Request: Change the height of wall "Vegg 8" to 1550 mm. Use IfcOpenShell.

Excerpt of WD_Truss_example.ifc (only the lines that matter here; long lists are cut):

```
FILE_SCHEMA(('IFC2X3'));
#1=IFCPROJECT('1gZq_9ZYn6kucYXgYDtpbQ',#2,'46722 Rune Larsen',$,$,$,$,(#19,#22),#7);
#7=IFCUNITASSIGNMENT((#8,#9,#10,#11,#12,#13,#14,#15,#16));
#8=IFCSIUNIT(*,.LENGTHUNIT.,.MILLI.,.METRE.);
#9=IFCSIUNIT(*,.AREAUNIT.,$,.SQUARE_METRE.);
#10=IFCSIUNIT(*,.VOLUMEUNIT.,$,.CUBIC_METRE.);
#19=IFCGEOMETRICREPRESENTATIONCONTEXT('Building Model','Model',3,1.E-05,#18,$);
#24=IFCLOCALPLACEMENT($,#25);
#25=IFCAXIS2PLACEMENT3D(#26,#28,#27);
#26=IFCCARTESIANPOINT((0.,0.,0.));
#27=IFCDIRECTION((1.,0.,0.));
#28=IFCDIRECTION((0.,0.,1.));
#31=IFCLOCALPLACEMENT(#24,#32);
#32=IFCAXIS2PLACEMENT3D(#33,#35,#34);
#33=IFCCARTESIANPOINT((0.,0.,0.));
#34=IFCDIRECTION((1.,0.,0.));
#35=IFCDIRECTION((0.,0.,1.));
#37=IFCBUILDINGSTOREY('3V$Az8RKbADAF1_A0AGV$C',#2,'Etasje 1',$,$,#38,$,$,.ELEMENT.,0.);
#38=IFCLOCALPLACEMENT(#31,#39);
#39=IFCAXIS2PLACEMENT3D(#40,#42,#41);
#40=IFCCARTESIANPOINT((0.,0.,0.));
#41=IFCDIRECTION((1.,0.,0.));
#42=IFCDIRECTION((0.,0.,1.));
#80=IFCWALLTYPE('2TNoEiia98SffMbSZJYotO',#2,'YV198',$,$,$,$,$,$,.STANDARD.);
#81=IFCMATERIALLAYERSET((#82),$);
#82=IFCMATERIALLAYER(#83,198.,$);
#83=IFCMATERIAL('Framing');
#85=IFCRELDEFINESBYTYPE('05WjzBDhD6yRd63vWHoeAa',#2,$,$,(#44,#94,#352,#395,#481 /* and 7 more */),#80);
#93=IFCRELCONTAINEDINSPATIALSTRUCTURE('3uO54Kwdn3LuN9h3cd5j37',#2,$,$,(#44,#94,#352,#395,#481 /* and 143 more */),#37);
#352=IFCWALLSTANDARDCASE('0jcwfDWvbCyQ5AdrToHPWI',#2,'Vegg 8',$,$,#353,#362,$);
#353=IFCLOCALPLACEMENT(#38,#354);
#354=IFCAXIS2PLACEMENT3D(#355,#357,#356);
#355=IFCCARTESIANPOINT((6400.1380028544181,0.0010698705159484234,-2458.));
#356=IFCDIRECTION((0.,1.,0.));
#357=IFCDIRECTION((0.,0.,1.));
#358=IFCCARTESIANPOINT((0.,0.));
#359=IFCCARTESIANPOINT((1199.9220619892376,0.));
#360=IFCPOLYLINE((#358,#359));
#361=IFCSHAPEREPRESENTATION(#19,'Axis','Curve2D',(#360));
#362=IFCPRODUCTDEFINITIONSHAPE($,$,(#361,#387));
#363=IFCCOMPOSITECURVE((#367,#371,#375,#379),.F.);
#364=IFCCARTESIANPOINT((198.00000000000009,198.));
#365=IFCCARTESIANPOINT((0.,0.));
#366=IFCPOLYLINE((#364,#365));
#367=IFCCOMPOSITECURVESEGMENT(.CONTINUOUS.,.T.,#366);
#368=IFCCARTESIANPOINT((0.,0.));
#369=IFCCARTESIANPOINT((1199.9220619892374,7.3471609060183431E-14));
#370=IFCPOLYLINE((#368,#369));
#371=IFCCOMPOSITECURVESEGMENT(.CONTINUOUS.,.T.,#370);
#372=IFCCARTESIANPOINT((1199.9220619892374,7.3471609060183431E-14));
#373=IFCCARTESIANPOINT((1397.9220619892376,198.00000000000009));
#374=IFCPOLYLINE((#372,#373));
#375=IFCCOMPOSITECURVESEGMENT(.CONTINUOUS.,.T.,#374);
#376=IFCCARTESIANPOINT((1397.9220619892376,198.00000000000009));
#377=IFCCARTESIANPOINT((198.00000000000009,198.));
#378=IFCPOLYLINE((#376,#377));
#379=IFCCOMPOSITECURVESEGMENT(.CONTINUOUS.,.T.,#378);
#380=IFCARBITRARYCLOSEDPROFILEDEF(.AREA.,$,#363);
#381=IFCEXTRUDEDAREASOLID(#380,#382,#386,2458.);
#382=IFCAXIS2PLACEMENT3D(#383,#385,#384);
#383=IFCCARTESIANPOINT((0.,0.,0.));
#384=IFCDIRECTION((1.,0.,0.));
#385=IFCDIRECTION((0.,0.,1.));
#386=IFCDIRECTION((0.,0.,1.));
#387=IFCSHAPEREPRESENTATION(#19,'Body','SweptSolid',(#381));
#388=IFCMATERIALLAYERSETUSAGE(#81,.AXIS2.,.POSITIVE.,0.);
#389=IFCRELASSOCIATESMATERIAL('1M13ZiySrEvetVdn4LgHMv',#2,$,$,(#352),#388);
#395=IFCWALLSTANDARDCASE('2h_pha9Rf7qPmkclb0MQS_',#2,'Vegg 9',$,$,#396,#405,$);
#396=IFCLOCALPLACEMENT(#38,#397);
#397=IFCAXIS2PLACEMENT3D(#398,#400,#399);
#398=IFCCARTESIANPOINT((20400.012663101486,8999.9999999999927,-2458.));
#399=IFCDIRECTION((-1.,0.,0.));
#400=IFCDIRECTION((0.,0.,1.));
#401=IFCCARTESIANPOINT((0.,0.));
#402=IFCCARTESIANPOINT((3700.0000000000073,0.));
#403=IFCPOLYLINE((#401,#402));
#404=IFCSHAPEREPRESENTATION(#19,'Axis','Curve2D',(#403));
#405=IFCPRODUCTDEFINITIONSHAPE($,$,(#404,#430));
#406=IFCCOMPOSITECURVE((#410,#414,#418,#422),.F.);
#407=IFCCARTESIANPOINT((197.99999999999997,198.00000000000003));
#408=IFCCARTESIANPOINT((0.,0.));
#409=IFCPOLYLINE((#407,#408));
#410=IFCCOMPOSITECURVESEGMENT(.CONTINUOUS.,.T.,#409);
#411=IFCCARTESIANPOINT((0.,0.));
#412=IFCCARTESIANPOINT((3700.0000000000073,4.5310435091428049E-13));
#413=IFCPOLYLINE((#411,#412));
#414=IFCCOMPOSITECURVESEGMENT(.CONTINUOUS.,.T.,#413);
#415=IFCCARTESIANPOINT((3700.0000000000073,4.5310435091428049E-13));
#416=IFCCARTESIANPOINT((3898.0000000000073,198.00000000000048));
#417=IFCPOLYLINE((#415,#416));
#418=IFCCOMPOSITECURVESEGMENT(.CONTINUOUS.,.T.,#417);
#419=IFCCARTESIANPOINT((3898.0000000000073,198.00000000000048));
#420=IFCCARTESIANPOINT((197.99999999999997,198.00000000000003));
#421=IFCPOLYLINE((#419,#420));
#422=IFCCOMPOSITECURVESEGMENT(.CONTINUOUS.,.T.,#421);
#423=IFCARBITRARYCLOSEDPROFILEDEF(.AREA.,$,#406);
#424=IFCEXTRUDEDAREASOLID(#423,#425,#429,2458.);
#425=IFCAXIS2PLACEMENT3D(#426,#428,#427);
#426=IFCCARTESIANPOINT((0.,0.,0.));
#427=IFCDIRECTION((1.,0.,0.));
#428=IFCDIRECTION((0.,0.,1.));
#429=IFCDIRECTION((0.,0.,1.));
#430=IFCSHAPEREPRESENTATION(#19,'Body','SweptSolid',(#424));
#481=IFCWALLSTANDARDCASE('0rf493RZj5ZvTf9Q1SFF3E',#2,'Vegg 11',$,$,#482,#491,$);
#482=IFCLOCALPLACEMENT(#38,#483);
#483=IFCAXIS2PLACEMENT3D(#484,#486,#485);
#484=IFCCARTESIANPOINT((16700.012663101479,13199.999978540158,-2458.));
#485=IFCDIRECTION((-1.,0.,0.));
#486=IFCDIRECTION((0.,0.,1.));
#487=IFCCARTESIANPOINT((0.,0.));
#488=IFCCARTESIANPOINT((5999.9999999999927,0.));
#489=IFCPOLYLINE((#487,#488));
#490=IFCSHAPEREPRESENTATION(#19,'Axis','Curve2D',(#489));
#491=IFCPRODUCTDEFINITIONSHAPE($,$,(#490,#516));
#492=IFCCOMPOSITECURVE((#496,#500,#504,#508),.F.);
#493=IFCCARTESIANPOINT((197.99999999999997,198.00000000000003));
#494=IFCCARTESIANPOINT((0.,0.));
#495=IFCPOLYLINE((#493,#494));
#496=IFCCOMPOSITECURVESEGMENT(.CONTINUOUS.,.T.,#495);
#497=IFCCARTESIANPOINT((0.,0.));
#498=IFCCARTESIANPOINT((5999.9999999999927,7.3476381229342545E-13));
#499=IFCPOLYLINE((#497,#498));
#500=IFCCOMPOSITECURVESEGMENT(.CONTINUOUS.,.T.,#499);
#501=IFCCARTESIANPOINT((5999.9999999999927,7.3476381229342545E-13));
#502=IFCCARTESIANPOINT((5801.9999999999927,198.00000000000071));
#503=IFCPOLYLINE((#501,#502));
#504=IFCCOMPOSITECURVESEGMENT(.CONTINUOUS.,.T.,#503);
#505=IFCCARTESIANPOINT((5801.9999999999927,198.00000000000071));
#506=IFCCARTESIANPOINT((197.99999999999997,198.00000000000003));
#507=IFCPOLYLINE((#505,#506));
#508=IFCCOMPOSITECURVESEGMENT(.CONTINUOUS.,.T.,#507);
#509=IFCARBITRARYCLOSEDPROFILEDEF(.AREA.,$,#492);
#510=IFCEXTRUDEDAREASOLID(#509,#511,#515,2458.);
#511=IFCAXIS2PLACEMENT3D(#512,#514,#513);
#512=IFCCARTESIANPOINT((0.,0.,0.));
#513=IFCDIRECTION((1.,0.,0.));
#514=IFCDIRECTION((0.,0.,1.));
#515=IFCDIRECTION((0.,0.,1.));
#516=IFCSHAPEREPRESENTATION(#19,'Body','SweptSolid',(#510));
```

```python
import ifcopenshell
import ifcopenshell.geom
import ifcopenshell.util.shape
import ifcopenshell.util.unit

model = ifcopenshell.open("WD_Truss_example.ifc")
unit_scale = ifcopenshell.util.unit.calculate_unit_scale(model)
settings = ifcopenshell.geom.settings()


def volume(element):
    """Net volume in cubic metres, openings subtracted."""
    shape = ifcopenshell.geom.create_shape(settings, element)
    return ifcopenshell.util.shape.get_volume(shape.geometry)


wall = model.by_guid("0jcwfDWvbCyQ5AdrToHPWI")
before = volume(wall)

body = next(r for r in wall.Representation.Representations if r.RepresentationIdentifier == "Body")
solid = body.Items[0]
old_height = solid.Depth
solid.Depth = 1.55 / unit_scale
after = volume(wall)

print(f"height {old_height:g} -> {solid.Depth:g}, volume {before:.3f} -> {after:.3f} m3")

model.write("WD_Truss_example-out.ifc")
```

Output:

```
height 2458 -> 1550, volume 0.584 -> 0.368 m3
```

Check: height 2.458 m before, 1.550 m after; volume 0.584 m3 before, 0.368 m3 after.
